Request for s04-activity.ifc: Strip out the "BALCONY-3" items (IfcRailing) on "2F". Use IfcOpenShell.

First a look at what the model holds.

```python
import ifcopenshell
import ifcopenshell.util.element

model = ifcopenshell.open("s04-activity.ifc")
print(model.schema)
storey = next(s for s in model.by_type("IfcBuildingStorey") if s.Name == "2F")
railings = [e for e in ifcopenshell.util.element.get_decomposition(storey) if e.is_a("IfcRailing")]
seen = {}
for e in railings:
    element_type = ifcopenshell.util.element.get_type(e)
    name = element_type.Name if element_type not in (None, e) else None
    seen[name] = seen.get(name, 0) + 1
for name, count in sorted(seen.items(), key=str):
    print(count, "x", name)
```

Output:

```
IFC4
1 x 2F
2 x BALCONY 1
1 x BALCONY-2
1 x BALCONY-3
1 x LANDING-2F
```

```python
import ifcopenshell
import ifcopenshell.api.root
import ifcopenshell.util.element

model = ifcopenshell.open("s04-activity.ifc")

storey = next(s for s in model.by_type("IfcBuildingStorey") if s.Name == "2F")
railings = [e for e in ifcopenshell.util.element.get_decomposition(storey) if e.is_a("IfcRailing")]
targets = [e for e in railings if (t := ifcopenshell.util.element.get_type(e)) not in (None, e) and t.Name == "BALCONY-3"]

for e in targets:
    ifcopenshell.api.root.remove_product(model, product=e)
print(len(targets), "removed")

model.write("s04-activity_edited.ifc")
```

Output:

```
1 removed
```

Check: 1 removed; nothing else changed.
